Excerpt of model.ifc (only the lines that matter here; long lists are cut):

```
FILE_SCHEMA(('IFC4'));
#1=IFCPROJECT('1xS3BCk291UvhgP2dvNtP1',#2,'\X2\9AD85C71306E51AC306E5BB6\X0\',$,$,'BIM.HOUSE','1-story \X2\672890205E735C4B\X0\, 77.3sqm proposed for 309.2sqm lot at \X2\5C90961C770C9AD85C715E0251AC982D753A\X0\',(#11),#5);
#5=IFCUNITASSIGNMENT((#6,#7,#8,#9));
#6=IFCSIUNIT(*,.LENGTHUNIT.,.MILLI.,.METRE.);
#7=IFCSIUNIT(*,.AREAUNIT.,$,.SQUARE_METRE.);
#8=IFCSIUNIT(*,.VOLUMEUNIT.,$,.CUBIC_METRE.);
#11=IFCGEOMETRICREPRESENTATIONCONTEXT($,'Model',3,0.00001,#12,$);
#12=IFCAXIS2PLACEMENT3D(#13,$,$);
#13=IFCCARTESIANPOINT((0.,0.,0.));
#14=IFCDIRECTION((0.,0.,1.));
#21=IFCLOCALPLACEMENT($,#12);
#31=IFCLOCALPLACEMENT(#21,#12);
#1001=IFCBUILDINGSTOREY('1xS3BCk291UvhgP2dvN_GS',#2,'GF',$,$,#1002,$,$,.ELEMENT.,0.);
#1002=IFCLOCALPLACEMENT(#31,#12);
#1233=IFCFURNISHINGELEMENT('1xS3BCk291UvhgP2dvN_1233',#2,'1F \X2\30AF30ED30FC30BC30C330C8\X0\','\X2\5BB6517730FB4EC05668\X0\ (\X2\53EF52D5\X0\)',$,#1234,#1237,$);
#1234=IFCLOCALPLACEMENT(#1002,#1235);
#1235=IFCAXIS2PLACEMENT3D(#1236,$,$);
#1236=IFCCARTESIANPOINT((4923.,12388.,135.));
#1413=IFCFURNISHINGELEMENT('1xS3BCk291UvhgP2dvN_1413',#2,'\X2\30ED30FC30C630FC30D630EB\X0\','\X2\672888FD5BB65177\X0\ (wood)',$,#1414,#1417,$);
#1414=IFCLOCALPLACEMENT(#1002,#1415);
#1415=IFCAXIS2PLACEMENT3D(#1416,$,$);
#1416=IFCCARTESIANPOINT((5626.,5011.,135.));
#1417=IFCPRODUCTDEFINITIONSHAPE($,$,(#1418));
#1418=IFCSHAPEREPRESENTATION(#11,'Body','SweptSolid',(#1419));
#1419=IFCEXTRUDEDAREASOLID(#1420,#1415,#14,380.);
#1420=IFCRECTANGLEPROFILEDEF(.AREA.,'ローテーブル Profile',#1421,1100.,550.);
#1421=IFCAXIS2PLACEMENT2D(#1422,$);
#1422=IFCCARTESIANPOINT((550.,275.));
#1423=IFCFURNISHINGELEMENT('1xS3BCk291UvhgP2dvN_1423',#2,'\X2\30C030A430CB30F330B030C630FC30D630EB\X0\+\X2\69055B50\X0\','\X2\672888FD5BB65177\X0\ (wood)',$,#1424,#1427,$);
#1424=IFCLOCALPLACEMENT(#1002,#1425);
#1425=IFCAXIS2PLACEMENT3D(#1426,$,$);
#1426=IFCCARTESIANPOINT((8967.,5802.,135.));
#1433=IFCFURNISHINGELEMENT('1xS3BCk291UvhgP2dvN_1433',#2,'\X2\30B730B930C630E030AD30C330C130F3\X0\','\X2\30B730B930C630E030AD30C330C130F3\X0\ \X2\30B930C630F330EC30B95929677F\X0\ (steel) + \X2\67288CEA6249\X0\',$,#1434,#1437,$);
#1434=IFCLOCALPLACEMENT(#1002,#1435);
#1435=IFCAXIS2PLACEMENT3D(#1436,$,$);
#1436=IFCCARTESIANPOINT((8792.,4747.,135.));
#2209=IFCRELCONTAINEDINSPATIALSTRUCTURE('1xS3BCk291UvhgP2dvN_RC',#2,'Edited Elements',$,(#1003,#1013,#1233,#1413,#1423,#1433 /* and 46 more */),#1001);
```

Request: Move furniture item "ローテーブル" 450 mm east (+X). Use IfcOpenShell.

```python
import ifcopenshell
import ifcopenshell.api.geometry
import ifcopenshell.util.placement

model = ifcopenshell.open("model.ifc")

item = model.by_id(1413)
matrix = ifcopenshell.util.placement.get_local_placement(item.ObjectPlacement)
matrix[0, 3] += 450.0
ifcopenshell.api.geometry.edit_object_placement(model, product=item, matrix=matrix, is_si=False)

print(ifcopenshell.util.placement.get_local_placement(item.ObjectPlacement).round(3) + 0.0)

model.write("model_updated.ifc")
```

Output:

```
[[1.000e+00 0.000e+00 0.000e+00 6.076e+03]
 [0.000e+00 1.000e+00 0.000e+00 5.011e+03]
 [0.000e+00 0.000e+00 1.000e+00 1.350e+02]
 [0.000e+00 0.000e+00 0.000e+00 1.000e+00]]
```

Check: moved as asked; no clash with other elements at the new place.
